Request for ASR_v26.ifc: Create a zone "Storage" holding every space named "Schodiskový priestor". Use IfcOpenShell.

First a look at what the model holds.

```python
import ifcopenshell

model = ifcopenshell.open("ASR_v26.ifc")
print(model.schema)
seen = {}
for space in model.by_type("IfcSpace"):
    seen[space.LongName] = seen.get(space.LongName, 0) + 1
for name, count in sorted(seen.items(), key=str):
    print(count, "x", name)
print("zones:", [z.Name for z in model.by_type("IfcZone")][:20])
```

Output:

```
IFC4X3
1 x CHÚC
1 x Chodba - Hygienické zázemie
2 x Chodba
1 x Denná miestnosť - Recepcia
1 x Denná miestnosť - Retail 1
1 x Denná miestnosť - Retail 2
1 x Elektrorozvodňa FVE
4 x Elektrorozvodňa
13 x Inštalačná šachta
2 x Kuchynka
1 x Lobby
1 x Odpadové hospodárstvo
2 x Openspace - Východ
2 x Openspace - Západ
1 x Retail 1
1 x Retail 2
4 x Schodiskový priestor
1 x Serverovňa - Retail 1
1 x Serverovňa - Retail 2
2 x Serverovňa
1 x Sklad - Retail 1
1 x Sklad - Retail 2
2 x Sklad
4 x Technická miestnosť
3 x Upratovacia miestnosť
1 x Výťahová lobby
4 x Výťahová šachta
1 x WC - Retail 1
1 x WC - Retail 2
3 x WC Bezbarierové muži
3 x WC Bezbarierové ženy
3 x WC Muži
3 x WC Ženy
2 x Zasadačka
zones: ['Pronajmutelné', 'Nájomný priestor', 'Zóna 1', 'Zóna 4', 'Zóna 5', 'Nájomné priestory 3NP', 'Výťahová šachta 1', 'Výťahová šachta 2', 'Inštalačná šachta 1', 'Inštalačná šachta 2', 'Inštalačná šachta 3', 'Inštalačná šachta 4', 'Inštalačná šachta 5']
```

```python
import ifcopenshell
import ifcopenshell.api.group
import ifcopenshell.api.root

model = ifcopenshell.open("ASR_v26.ifc")

names = {"Schodiskový priestor"}
spaces = [s for s in model.by_type("IfcSpace") if s.LongName in names]

zone = ifcopenshell.api.root.create_entity(model, ifc_class="IfcZone", name="Storage")
ifcopenshell.api.group.assign_group(model, products=spaces, group=zone)
print(len(spaces), "spaces in", zone.Name)

model.write("ASR_v26_rev.ifc")
```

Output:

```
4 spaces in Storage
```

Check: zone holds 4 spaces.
